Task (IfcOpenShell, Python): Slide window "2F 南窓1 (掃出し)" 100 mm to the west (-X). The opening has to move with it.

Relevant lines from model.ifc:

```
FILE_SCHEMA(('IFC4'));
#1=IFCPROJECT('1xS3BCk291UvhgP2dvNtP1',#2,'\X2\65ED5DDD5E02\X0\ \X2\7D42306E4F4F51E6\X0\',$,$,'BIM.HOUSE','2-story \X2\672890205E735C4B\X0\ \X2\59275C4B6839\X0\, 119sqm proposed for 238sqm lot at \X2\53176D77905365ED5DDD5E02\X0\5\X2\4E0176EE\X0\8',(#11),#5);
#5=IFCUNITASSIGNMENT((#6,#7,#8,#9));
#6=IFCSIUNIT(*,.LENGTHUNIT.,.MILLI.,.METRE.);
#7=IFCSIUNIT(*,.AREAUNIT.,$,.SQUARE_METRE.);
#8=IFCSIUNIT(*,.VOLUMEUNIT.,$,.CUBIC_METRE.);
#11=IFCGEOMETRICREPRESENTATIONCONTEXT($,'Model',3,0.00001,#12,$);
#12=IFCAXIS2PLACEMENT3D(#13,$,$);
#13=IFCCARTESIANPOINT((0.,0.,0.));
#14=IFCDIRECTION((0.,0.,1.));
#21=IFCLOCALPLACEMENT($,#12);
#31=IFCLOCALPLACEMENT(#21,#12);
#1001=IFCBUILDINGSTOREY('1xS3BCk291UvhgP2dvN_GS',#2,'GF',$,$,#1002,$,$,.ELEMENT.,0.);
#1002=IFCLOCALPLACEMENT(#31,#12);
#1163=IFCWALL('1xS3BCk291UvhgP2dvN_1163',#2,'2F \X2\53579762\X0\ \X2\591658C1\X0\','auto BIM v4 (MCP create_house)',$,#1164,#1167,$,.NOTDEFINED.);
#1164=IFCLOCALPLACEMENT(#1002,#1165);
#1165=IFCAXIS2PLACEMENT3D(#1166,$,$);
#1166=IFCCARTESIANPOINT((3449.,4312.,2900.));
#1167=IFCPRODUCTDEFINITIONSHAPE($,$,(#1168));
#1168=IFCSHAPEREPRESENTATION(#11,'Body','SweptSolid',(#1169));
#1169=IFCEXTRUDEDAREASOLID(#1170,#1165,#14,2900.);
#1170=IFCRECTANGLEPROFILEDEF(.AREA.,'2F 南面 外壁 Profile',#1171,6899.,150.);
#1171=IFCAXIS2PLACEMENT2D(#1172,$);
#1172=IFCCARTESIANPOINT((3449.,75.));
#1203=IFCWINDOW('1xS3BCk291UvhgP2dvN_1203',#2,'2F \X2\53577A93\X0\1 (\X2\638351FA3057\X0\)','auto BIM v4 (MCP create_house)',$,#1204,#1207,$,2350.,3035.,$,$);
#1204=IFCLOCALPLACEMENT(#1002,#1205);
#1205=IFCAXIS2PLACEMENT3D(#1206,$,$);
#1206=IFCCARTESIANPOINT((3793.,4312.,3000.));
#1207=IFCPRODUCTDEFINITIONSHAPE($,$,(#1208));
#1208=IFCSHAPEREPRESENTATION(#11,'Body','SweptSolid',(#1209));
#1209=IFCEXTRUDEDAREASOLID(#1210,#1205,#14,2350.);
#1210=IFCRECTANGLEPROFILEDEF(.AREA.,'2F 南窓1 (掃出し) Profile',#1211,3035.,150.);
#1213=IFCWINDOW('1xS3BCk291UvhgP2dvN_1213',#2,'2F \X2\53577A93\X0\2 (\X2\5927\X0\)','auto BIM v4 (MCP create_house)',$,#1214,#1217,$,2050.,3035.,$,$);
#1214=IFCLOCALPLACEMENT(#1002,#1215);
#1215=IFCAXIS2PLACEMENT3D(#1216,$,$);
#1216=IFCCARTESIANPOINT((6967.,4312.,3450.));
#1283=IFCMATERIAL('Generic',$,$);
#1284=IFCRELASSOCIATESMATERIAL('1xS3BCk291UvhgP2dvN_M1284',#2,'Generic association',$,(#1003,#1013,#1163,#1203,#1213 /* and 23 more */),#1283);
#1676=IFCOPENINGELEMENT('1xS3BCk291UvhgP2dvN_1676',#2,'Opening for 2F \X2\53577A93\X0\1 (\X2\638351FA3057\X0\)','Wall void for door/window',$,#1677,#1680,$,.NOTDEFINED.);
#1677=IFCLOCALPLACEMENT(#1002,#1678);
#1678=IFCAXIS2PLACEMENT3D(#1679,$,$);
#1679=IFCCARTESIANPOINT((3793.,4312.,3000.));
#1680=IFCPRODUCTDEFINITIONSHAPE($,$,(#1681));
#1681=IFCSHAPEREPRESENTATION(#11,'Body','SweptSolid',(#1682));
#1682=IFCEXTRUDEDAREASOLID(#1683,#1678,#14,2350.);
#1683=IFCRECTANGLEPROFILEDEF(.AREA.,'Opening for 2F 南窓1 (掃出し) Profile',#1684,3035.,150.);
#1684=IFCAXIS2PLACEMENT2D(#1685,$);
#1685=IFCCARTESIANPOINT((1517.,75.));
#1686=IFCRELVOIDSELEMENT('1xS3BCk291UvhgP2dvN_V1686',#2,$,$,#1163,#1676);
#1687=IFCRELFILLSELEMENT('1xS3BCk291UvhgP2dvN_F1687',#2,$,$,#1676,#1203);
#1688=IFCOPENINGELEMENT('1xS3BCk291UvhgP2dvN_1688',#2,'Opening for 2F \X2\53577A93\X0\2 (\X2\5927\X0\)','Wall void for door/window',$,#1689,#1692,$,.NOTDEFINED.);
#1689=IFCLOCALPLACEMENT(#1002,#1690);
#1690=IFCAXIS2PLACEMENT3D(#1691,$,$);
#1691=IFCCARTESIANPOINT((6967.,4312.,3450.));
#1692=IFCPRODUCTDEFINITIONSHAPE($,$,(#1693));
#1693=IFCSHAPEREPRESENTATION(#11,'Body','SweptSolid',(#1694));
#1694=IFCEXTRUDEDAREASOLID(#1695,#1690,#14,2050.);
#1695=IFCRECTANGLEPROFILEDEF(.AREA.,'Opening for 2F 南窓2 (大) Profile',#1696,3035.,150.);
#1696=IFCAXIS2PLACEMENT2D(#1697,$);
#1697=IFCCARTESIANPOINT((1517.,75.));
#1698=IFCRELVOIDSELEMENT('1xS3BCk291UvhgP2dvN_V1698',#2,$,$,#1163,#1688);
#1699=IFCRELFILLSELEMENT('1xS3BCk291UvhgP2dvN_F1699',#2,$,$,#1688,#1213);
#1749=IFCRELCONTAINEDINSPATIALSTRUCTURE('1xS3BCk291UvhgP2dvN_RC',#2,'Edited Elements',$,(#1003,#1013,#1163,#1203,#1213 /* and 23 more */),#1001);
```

```python
import ifcopenshell
import ifcopenshell.api.geometry
import ifcopenshell.util.placement
import ifcopenshell.util.unit

model = ifcopenshell.open("model.ifc")
unit_scale = ifcopenshell.util.unit.calculate_unit_scale(model)

window = model.by_guid("1xS3BCk291UvhgP2dvN_1203")
opening = window.FillsVoids[0].RelatingOpeningElement
wall = opening.VoidsElements[0].RelatingBuildingElement

wall_matrix = ifcopenshell.util.placement.get_local_placement(wall.ObjectPlacement)
shift = wall_matrix[:3, 0] * -0.1 / unit_scale
before = ifcopenshell.util.placement.get_local_placement(window.ObjectPlacement)[:3, 3].copy()

# The window is not placed relative to its opening, so move both.
for product in (opening, window):
    matrix = ifcopenshell.util.placement.get_local_placement(product.ObjectPlacement)
    matrix[:3, 3] += shift
    ifcopenshell.api.geometry.edit_object_placement(model, product=product, matrix=matrix, is_si=False)

after = ifcopenshell.util.placement.get_local_placement(window.ObjectPlacement)[:3, 3]
print("window moved by", (after - before).round(3) + 0.0)

model.write("model-out.ifc")
```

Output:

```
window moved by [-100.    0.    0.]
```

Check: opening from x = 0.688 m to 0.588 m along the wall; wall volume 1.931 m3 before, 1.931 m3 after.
